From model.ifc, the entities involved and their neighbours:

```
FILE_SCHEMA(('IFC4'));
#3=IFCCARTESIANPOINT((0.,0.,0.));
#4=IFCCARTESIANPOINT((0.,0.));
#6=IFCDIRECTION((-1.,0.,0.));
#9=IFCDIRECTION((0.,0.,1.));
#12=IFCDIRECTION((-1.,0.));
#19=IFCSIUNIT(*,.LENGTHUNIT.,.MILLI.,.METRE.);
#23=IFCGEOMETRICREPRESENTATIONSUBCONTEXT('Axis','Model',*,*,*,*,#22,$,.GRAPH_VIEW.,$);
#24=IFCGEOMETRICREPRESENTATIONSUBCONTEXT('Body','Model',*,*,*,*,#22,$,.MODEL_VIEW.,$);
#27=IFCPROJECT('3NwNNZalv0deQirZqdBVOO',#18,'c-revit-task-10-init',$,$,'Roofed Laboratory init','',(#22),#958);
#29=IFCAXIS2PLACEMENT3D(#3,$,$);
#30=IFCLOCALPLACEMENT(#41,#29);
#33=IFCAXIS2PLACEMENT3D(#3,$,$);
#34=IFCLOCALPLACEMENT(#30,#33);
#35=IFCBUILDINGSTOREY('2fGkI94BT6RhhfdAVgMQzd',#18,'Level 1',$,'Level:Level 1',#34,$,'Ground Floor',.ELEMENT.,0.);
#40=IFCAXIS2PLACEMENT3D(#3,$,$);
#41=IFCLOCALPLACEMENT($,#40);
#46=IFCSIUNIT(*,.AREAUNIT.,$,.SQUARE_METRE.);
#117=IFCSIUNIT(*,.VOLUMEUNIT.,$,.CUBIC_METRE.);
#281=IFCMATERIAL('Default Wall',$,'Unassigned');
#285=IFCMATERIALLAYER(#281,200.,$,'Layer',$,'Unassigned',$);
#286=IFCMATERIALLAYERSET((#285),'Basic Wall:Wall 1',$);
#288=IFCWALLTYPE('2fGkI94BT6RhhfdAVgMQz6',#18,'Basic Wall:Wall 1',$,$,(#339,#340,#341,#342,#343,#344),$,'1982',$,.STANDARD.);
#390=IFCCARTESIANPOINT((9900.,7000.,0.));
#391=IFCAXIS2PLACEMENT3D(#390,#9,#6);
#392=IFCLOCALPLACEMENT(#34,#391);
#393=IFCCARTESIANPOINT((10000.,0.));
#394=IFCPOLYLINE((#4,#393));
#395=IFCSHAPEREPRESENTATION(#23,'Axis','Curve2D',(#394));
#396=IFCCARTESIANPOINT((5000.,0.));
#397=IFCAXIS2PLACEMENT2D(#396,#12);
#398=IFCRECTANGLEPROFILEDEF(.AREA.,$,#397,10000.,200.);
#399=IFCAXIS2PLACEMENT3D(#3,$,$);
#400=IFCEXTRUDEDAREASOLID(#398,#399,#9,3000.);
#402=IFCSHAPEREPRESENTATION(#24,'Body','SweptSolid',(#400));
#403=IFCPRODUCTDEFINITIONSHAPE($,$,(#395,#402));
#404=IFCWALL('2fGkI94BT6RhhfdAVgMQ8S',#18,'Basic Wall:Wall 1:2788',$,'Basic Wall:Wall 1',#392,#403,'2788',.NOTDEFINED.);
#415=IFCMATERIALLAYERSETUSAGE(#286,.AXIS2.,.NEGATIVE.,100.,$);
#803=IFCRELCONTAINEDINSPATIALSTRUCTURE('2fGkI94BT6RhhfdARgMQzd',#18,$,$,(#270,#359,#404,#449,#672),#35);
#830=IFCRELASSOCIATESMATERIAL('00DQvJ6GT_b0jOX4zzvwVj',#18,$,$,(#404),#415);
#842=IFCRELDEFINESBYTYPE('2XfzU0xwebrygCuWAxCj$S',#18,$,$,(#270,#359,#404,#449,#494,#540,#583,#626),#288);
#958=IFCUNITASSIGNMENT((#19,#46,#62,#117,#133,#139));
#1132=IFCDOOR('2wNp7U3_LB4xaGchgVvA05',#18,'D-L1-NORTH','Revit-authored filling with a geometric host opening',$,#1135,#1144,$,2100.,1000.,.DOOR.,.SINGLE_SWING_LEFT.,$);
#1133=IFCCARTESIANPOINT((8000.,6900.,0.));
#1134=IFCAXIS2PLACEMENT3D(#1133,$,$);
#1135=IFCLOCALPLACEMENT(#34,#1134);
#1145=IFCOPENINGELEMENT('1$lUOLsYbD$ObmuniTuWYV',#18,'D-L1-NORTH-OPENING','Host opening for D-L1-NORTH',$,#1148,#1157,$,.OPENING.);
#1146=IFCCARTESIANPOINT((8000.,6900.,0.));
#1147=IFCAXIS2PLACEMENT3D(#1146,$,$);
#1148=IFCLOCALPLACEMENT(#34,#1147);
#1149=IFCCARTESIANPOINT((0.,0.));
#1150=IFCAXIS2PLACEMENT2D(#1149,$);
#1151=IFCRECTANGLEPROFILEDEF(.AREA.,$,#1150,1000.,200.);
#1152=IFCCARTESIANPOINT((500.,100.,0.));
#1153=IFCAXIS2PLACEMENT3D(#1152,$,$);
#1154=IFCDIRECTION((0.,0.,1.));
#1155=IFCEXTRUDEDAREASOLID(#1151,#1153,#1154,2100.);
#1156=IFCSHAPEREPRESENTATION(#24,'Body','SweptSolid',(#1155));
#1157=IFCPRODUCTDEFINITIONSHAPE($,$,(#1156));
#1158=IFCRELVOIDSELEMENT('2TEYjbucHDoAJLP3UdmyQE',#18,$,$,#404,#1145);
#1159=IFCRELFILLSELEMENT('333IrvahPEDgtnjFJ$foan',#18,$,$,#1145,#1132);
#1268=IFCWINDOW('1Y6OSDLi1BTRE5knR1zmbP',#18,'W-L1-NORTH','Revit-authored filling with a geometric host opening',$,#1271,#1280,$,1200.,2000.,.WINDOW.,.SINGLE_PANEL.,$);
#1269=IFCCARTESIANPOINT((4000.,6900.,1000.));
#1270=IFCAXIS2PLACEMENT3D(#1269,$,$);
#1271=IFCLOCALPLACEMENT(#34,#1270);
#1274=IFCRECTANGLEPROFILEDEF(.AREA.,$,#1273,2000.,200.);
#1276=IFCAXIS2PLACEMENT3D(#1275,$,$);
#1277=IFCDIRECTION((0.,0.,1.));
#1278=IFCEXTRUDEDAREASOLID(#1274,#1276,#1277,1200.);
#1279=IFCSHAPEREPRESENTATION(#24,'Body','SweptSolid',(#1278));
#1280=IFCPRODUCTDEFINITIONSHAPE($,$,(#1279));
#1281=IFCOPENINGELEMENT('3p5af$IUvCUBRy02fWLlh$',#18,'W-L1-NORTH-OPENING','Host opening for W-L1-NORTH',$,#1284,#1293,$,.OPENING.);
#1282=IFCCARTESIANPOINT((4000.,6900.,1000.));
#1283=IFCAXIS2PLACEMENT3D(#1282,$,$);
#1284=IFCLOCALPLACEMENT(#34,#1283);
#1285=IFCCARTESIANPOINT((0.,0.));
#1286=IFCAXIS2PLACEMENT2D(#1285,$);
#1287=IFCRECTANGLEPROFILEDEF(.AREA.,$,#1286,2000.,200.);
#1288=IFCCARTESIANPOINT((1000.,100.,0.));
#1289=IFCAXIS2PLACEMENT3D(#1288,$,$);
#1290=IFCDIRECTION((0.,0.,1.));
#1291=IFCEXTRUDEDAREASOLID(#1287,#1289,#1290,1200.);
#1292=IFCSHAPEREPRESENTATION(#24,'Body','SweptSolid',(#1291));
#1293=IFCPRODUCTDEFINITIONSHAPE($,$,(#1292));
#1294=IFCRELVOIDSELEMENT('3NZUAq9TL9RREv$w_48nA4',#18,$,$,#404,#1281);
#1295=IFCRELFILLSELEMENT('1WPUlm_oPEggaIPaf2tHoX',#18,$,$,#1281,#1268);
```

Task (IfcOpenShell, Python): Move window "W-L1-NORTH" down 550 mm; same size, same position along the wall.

```python
import numpy as np
import ifcopenshell
import ifcopenshell.api.geometry
import ifcopenshell.util.placement
import ifcopenshell.util.unit

model = ifcopenshell.open("model.ifc")
unit_scale = ifcopenshell.util.unit.calculate_unit_scale(model)

window = model.by_id(1268)
opening = window.FillsVoids[0].RelatingOpeningElement
dz = -550.0

shift = np.array([0.0, 0.0, dz])
# The window is not placed relative to its opening, so move both.
for product in (opening, window):
    matrix = ifcopenshell.util.placement.get_local_placement(product.ObjectPlacement)
    matrix[:3, 3] += shift
    ifcopenshell.api.geometry.edit_object_placement(model, product=product, matrix=matrix, is_si=False)

print(f"moved by {dz * unit_scale:+.3f} m")

model.write("model_updated.ifc")
```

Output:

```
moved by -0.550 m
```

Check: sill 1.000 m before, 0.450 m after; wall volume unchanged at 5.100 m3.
